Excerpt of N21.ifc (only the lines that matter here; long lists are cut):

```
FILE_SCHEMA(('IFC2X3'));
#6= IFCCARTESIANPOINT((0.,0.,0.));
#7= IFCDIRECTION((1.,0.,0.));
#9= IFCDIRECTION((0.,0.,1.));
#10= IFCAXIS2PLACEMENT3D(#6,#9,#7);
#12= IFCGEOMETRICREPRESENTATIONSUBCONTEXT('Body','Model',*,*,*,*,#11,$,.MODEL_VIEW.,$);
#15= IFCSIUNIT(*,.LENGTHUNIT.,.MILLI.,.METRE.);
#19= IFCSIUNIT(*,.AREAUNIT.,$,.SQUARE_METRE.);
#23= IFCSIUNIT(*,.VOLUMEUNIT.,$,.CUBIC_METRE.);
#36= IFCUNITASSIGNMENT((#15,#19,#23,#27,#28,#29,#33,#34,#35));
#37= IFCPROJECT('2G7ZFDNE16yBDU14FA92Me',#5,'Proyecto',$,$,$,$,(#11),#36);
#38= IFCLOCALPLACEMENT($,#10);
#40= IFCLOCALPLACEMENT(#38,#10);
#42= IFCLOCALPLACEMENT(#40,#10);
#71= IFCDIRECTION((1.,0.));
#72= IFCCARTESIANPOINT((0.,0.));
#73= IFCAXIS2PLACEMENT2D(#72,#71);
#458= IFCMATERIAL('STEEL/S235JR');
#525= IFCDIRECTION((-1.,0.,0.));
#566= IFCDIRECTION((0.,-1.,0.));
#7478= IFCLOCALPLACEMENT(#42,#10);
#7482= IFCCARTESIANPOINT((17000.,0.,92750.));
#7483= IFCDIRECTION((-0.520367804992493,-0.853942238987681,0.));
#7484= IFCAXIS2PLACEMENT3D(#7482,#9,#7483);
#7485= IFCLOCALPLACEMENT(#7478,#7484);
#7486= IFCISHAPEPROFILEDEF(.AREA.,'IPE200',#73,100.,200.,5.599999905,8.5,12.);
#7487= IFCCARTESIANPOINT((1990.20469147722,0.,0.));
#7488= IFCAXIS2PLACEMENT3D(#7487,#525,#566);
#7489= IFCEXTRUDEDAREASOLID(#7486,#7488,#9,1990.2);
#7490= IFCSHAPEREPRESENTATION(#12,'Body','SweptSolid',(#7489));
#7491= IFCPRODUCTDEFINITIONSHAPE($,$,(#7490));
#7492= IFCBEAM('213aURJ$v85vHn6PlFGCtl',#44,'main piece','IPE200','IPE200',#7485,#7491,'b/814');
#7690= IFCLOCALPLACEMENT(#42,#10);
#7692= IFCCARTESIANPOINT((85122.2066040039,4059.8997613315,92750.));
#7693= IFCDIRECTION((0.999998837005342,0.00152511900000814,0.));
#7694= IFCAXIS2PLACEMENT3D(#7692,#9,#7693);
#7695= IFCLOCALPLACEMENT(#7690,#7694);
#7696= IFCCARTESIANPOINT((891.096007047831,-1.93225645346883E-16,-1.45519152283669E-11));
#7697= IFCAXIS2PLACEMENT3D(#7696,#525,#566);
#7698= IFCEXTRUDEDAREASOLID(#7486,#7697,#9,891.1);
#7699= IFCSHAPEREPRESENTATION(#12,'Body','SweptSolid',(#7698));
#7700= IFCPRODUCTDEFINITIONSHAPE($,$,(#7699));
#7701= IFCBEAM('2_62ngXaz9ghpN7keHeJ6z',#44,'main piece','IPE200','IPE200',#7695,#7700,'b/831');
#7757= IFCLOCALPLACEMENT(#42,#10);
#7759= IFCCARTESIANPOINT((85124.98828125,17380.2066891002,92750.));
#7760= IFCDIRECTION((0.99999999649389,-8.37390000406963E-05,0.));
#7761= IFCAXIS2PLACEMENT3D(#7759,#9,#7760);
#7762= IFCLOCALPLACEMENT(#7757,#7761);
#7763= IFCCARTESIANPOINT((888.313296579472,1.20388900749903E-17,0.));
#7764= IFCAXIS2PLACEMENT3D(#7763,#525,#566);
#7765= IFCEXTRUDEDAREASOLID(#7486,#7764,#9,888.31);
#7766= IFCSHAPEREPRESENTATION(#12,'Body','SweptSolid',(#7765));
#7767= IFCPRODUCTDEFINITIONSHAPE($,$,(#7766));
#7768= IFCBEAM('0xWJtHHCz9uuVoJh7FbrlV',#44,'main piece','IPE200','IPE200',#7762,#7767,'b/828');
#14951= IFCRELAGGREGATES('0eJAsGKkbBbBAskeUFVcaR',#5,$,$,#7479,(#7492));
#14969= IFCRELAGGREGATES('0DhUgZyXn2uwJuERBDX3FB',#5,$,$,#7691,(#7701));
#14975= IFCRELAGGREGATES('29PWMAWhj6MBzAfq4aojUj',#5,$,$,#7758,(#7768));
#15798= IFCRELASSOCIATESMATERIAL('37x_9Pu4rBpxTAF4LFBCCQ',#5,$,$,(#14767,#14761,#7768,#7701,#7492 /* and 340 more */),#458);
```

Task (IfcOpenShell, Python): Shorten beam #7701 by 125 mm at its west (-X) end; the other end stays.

```python
import ifcopenshell
import ifcopenshell.util.representation

model = ifcopenshell.open("N21.ifc")

member = model.by_guid("2_62ngXaz9ghpN7keHeJ6z")
change = -125.0

# The extrusion runs towards the end named, so only its depth changes.
body = ifcopenshell.util.representation.get_representation(member, "Model", "Body")
solid = body.Items[0]
old_length = solid.Depth
solid.Depth += change

print(f"length {old_length:g} -> {solid.Depth:g}")

model.write("N21_v2.ifc")
```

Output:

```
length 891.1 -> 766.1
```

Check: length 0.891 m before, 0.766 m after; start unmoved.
